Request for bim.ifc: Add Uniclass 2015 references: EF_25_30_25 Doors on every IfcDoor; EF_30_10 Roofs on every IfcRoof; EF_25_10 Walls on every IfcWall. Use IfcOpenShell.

First a look at what the model holds.

```python
import ifcopenshell

model = ifcopenshell.open("bim.ifc")
print(model.schema)
print("classifications:", [c.Name for c in model.by_type("IfcClassification")])
for ifc_class in ("IfcDoor", "IfcRoof", "IfcStair", "IfcWall", "IfcWindow"):
    print(ifc_class, len(model.by_type(ifc_class)))
```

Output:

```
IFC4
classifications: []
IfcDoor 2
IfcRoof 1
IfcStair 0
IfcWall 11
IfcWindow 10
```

```python
import ifcopenshell
import ifcopenshell.api.classification

model = ifcopenshell.open("bim.ifc")

system = ifcopenshell.api.classification.add_classification(model, classification="Uniclass 2015")

codes = {
    "IfcDoor": ("EF_25_30_25", "Doors"),
    "IfcRoof": ("EF_30_10", "Roofs"),
    "IfcWall": ("EF_25_10", "Walls"),
}
for ifc_class, (code, name) in codes.items():
    products = model.by_type(ifc_class)
    ifcopenshell.api.classification.add_reference(
        model, products=products, classification=system, identification=code, name=name
    )
    print(code, len(products))

model.write("bim-out.ifc")
```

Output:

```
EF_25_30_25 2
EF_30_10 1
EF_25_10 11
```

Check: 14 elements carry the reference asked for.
